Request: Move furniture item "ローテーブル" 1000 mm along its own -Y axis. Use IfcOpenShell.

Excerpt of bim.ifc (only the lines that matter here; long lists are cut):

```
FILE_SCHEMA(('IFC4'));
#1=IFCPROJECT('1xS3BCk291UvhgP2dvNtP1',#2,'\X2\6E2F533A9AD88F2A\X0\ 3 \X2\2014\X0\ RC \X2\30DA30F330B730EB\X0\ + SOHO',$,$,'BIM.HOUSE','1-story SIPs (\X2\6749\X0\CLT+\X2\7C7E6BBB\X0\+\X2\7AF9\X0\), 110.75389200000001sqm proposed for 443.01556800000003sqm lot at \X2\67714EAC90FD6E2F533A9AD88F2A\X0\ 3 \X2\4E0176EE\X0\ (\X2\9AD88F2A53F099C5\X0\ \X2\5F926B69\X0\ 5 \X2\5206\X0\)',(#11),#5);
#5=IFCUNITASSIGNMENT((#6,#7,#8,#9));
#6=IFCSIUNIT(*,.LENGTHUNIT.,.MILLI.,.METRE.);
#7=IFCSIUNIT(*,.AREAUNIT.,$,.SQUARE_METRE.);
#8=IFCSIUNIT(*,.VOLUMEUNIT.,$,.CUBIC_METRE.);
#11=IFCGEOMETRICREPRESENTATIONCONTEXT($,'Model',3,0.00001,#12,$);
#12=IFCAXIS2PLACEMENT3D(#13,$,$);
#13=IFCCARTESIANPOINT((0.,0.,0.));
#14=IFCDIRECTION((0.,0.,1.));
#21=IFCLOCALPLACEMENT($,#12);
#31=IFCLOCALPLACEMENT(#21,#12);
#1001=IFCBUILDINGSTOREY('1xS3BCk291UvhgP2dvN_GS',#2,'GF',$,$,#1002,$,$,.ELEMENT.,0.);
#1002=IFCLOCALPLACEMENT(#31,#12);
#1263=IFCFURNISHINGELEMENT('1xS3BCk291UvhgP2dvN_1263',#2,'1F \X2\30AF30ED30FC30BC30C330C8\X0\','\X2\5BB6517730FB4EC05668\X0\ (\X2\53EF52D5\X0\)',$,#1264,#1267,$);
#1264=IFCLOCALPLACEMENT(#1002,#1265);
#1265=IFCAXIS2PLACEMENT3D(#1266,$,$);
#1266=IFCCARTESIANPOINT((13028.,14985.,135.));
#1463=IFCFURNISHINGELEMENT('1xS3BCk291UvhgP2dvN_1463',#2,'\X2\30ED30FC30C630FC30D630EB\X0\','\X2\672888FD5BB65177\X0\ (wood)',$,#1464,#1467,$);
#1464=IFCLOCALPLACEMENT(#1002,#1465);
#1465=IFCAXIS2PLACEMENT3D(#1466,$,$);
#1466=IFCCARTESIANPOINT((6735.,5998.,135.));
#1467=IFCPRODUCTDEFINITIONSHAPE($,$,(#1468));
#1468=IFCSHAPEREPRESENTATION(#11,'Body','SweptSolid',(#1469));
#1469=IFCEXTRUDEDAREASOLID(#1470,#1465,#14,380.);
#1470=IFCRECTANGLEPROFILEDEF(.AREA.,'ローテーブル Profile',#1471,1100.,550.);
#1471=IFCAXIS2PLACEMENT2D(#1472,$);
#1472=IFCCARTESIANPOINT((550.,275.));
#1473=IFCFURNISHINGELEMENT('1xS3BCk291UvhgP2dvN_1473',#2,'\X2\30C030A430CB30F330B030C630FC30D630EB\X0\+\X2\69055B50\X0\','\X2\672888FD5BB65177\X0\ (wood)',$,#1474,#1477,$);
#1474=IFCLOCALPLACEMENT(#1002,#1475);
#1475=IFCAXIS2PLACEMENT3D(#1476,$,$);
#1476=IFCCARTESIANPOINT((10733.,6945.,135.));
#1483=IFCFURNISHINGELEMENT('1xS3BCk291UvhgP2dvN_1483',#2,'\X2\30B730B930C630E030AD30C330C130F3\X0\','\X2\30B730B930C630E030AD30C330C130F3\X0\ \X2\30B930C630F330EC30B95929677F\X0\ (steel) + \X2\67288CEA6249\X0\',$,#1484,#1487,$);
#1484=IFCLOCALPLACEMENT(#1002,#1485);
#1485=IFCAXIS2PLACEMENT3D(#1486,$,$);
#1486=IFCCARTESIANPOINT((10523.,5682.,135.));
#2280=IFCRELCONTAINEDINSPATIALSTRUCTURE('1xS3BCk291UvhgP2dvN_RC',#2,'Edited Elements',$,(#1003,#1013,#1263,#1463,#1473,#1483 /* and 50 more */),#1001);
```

```python
import ifcopenshell
import ifcopenshell.api.geometry
import ifcopenshell.util.placement
import ifcopenshell.util.unit

model = ifcopenshell.open("bim.ifc")
unit_scale = ifcopenshell.util.unit.calculate_unit_scale(model)

item = model.by_guid("1xS3BCk291UvhgP2dvN_1463")
matrix = ifcopenshell.util.placement.get_local_placement(item.ObjectPlacement)
matrix[:3, 3] -= matrix[:3, 1] * 1 / unit_scale
ifcopenshell.api.geometry.edit_object_placement(model, product=item, matrix=matrix, is_si=False)

print(ifcopenshell.util.placement.get_local_placement(item.ObjectPlacement).round(3) + 0.0)

model.write("bim_rev.ifc")
```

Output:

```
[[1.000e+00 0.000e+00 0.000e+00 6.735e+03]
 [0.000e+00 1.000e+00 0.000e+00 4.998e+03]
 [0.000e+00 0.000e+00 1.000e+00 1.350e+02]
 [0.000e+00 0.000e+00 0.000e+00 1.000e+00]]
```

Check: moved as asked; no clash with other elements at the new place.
